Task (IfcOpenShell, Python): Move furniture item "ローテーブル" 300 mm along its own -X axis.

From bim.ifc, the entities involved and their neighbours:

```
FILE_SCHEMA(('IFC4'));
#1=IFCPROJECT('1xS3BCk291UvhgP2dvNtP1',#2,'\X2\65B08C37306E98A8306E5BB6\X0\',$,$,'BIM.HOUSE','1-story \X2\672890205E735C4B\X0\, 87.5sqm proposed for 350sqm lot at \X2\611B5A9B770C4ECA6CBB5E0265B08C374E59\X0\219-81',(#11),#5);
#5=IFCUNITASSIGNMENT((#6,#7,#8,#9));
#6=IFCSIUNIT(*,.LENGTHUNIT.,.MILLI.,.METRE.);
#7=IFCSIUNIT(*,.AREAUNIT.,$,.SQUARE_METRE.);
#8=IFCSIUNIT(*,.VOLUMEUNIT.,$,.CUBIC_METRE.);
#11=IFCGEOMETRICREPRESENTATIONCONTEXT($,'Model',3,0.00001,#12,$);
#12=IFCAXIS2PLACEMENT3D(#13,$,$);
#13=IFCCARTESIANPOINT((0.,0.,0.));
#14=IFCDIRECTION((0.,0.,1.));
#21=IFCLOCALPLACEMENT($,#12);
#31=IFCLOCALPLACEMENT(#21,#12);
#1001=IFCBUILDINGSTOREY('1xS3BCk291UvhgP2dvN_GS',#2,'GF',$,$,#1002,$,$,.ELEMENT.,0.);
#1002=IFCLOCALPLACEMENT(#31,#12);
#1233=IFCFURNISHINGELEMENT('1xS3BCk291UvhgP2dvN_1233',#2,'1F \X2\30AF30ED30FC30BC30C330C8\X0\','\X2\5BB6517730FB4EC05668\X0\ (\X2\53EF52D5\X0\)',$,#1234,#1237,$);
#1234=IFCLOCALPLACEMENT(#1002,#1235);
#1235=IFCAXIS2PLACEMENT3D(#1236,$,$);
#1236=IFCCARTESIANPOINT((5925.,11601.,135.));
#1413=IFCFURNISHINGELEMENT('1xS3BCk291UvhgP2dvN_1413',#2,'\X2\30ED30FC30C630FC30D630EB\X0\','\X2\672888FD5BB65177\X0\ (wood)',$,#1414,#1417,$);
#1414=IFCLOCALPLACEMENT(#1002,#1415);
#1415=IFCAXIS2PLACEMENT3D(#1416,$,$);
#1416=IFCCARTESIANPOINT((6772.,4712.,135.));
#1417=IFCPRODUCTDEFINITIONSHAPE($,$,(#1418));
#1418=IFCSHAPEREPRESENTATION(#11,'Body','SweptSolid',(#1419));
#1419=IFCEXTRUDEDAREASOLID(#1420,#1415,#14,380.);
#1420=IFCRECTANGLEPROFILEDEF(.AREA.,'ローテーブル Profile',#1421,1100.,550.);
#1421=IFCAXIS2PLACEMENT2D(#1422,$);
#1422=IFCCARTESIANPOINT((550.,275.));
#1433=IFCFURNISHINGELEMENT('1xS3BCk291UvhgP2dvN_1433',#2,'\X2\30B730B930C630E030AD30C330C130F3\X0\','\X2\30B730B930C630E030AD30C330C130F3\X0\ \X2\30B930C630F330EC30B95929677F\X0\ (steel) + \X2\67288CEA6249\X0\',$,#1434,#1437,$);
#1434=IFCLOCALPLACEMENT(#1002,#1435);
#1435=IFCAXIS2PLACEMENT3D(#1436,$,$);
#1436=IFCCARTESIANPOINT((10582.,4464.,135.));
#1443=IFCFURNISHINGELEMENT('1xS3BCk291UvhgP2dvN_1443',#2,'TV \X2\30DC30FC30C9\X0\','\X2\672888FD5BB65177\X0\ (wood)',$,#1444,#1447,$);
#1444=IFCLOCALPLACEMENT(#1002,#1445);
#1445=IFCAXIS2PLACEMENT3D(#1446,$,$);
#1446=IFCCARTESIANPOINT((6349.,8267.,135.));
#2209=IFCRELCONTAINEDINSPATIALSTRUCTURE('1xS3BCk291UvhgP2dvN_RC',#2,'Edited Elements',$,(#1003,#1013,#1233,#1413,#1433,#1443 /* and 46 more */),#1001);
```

```python
import ifcopenshell
import ifcopenshell.api.geometry
import ifcopenshell.util.placement
import ifcopenshell.util.unit

model = ifcopenshell.open("bim.ifc")
unit_scale = ifcopenshell.util.unit.calculate_unit_scale(model)

item = model.by_guid("1xS3BCk291UvhgP2dvN_1413")
matrix = ifcopenshell.util.placement.get_local_placement(item.ObjectPlacement)
matrix[:3, 3] -= matrix[:3, 0] * 0.3 / unit_scale
ifcopenshell.api.geometry.edit_object_placement(model, product=item, matrix=matrix, is_si=False)

print(ifcopenshell.util.placement.get_local_placement(item.ObjectPlacement).round(3) + 0.0)

model.write("bim_v2.ifc")
```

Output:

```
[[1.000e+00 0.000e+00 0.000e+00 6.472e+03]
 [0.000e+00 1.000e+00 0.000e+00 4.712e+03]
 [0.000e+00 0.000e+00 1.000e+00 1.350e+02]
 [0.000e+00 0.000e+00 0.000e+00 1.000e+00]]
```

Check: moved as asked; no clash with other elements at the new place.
